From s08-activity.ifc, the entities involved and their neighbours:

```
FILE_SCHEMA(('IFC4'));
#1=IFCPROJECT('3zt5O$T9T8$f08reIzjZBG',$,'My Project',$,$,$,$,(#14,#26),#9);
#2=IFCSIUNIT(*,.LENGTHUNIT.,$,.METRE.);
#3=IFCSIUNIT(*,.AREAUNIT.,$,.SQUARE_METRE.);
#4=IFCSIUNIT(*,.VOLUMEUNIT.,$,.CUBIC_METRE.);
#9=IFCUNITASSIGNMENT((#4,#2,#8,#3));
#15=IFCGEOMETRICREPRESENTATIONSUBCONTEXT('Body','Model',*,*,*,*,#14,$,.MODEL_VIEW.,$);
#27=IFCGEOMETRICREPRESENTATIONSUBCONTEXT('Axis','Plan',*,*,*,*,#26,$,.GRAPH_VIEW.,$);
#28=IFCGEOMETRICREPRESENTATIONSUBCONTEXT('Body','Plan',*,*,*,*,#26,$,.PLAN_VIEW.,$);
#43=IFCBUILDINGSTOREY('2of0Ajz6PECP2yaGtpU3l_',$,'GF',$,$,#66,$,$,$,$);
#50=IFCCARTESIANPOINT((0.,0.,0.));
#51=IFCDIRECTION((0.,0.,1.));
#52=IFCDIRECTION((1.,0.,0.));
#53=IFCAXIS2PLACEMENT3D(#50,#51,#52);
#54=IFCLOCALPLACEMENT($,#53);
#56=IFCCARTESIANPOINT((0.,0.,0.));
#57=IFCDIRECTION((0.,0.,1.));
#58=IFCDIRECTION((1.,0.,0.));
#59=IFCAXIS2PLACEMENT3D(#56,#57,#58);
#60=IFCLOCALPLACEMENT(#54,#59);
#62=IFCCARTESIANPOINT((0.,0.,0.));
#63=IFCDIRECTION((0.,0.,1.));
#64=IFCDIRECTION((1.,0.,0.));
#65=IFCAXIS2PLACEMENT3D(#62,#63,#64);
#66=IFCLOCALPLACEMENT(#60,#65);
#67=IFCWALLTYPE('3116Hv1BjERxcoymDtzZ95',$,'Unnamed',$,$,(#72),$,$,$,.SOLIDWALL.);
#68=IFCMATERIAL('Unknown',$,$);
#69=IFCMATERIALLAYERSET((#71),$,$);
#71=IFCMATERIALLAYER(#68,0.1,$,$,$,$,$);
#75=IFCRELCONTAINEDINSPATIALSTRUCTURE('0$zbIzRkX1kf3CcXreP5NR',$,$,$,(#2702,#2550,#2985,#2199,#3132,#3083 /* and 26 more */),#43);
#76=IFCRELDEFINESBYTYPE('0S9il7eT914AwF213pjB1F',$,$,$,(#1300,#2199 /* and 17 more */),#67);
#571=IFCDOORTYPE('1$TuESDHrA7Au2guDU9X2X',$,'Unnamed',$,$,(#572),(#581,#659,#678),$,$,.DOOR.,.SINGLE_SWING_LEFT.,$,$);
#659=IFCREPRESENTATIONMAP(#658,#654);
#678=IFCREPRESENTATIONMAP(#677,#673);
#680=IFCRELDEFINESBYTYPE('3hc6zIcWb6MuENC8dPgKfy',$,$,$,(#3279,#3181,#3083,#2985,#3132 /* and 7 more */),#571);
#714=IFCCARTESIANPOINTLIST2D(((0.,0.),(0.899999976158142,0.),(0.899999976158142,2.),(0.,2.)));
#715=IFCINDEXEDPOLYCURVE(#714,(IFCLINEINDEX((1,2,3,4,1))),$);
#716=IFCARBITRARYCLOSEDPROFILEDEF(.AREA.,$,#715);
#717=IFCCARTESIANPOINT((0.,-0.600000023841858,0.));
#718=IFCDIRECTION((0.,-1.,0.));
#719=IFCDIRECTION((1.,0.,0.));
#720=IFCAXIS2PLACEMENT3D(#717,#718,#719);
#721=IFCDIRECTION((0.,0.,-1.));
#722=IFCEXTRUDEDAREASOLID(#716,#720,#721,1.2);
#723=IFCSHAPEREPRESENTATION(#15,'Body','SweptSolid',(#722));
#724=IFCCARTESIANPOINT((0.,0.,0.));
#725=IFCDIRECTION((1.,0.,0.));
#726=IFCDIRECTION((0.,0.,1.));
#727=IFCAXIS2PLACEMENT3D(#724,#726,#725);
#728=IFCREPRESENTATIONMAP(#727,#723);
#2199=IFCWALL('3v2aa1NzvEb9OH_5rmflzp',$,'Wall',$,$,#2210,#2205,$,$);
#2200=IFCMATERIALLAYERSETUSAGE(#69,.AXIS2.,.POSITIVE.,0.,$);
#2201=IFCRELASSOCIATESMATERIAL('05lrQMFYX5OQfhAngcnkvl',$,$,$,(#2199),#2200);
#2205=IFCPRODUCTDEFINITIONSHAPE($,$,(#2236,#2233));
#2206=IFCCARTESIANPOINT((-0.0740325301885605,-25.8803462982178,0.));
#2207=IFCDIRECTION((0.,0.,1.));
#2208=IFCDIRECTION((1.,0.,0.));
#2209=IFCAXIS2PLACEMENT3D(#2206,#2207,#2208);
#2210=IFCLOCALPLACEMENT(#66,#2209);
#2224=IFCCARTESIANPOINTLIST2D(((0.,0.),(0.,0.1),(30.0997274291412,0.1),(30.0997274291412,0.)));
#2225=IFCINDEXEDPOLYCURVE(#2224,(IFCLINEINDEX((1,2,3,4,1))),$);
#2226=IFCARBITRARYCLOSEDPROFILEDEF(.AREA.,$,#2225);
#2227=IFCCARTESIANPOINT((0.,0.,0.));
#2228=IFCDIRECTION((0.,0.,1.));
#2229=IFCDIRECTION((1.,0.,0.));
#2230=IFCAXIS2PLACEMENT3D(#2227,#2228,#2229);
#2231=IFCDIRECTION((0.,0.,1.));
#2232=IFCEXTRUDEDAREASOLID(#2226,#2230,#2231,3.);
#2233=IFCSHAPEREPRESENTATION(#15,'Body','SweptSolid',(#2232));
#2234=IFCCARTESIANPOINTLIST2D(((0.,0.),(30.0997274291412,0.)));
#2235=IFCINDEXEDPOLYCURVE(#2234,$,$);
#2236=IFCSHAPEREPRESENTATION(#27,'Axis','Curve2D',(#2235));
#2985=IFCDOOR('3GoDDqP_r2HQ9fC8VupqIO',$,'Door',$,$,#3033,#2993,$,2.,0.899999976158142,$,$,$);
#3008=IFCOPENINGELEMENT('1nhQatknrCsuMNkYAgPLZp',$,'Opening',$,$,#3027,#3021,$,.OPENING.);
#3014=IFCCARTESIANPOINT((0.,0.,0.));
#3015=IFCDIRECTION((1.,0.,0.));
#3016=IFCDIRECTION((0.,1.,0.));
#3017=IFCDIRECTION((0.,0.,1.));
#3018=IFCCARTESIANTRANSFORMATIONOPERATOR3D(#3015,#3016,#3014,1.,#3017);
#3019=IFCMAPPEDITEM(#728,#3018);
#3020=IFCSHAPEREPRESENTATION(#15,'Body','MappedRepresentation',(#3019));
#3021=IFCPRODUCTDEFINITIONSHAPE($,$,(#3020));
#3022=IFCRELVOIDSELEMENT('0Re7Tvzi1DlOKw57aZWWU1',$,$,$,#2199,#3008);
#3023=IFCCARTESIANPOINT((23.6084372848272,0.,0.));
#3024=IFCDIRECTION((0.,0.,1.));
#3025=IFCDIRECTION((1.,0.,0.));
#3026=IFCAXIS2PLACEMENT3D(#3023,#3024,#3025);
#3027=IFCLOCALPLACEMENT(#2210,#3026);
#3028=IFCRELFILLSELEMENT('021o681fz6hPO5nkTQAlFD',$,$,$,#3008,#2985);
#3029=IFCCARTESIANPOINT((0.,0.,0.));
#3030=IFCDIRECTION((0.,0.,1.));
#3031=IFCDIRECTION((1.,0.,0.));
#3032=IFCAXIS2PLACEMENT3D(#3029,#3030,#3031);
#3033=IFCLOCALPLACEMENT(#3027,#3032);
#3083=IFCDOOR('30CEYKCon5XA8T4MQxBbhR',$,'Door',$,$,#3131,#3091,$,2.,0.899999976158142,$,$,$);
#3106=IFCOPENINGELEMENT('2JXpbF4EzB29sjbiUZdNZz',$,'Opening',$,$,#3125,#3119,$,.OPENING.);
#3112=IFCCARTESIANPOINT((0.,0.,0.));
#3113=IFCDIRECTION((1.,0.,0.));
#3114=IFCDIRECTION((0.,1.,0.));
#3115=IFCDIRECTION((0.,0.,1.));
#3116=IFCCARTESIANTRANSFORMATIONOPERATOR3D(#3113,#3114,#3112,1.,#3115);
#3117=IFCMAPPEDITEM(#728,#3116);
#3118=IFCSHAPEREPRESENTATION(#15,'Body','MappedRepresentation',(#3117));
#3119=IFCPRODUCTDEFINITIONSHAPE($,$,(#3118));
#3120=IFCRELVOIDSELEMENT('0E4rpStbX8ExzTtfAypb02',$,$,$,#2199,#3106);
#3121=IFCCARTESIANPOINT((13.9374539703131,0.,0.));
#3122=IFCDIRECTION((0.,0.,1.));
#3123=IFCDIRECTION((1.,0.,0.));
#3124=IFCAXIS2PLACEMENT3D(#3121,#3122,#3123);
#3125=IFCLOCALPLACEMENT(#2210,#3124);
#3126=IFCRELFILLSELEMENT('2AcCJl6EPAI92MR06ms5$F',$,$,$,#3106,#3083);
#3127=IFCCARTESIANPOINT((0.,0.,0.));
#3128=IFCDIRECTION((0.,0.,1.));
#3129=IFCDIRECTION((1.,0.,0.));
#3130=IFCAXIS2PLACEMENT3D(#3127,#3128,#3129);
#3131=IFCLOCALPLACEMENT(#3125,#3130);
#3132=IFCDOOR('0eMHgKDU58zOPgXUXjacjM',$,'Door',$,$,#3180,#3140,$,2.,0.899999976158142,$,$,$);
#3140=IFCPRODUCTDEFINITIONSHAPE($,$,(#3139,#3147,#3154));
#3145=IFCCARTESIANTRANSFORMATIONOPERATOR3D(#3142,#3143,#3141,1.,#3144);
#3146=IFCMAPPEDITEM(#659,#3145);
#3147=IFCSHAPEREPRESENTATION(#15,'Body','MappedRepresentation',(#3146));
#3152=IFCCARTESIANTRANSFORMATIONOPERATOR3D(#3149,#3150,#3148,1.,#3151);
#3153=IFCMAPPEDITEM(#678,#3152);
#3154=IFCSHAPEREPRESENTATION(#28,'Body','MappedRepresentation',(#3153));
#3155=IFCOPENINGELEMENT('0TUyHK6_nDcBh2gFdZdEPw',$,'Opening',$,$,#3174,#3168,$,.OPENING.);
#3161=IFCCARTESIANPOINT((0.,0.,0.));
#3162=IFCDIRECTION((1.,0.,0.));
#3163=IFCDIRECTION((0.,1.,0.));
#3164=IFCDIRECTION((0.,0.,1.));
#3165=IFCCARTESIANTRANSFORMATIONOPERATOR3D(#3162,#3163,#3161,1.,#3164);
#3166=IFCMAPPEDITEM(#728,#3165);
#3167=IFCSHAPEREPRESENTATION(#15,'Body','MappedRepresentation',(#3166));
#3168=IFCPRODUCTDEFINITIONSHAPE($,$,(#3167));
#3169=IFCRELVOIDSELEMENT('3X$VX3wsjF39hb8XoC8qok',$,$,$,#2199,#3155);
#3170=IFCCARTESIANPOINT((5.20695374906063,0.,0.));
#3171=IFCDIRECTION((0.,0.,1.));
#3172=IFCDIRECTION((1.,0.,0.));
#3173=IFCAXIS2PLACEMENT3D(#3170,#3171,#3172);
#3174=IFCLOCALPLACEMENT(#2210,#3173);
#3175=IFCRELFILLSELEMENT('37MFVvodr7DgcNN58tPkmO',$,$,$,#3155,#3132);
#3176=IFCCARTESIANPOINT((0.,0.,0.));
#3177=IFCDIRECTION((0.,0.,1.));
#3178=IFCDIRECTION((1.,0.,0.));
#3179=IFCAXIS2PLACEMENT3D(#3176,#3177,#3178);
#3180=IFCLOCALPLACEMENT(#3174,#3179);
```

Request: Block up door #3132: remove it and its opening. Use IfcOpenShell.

```python
import ifcopenshell
import ifcopenshell.api.feature
import ifcopenshell.api.root
import ifcopenshell.geom
import ifcopenshell.util.shape

model = ifcopenshell.open("s08-activity.ifc")
settings = ifcopenshell.geom.settings()


def volume(element):
    """Net volume in cubic metres, openings subtracted."""
    shape = ifcopenshell.geom.create_shape(settings, element)
    return ifcopenshell.util.shape.get_volume(shape.geometry)


door = model.by_id(3132)
opening = door.FillsVoids[0].RelatingOpeningElement
wall = opening.VoidsElements[0].RelatingBuildingElement
before = volume(wall)

ifcopenshell.api.root.remove_product(model, product=door)
ifcopenshell.api.feature.remove_feature(model, feature=opening)

after = volume(wall)

print(f"wall volume {before:.3f} -> {after:.3f} m3")

model.write("s08-activity-out.ifc")
```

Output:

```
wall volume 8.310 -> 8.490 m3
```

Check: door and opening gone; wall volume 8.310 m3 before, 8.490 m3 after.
